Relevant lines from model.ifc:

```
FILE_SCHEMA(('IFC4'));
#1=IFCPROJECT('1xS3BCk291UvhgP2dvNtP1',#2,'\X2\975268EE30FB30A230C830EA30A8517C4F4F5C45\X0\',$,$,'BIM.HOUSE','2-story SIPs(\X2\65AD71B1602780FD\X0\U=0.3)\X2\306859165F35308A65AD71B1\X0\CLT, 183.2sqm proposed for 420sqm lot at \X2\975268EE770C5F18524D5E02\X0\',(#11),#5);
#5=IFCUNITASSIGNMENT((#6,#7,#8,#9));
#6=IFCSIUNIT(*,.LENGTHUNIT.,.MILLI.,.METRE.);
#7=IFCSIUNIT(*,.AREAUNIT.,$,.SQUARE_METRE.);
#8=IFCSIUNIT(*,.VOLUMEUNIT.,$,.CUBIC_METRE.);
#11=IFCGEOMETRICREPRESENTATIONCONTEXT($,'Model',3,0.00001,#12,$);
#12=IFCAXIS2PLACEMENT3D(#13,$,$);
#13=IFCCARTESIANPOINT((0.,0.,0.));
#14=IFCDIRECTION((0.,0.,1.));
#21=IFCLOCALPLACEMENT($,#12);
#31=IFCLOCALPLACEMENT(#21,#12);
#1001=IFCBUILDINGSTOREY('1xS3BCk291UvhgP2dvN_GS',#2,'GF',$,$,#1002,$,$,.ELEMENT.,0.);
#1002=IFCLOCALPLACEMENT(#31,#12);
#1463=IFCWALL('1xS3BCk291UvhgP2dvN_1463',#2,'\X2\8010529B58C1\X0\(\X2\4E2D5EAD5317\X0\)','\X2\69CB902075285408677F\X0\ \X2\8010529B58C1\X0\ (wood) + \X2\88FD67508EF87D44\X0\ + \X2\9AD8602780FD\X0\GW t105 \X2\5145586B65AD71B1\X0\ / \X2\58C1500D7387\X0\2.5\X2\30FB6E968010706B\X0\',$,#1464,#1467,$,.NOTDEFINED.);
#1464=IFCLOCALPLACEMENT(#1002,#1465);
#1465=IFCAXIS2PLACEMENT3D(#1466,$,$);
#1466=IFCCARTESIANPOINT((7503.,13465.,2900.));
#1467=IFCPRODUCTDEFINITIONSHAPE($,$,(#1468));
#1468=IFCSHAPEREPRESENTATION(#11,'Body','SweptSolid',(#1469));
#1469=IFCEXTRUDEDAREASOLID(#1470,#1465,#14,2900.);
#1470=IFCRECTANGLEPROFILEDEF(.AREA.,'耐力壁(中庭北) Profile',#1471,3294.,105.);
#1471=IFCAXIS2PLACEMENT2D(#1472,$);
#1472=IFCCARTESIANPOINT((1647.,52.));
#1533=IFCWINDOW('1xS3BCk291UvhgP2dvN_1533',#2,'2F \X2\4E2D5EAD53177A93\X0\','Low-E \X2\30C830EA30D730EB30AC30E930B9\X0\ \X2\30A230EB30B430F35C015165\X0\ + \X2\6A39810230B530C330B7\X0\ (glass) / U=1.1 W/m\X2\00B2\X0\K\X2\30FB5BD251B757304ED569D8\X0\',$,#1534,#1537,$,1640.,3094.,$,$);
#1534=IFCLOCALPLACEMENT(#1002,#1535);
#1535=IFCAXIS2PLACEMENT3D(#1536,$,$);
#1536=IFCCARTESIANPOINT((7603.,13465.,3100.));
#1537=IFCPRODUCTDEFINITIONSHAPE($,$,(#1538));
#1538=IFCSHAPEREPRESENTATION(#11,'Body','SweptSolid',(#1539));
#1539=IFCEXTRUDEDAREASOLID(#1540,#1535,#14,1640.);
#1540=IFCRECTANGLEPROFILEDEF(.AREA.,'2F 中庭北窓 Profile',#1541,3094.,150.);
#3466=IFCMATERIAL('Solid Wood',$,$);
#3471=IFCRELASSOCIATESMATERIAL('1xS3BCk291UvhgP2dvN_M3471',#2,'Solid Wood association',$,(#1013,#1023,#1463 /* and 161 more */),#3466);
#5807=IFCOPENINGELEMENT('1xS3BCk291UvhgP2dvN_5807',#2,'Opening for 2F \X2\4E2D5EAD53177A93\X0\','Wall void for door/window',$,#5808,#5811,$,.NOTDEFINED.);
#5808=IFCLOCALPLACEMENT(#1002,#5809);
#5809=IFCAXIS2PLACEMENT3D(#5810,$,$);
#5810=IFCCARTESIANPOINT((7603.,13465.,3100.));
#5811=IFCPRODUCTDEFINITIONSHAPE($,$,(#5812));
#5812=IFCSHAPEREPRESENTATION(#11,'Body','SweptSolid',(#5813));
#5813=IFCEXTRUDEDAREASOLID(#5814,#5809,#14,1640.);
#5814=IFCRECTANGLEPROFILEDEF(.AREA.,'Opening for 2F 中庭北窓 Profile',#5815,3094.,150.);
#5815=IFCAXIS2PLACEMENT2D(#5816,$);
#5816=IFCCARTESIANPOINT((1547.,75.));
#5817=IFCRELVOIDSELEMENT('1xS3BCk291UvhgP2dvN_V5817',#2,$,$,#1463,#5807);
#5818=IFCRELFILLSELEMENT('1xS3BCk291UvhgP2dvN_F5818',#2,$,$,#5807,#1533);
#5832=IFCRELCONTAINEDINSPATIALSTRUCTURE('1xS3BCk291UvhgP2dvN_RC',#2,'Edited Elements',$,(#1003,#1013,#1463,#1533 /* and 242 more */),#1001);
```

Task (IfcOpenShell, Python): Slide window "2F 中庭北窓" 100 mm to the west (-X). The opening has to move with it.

```python
import ifcopenshell
import ifcopenshell.api.geometry
import ifcopenshell.util.placement
import ifcopenshell.util.unit

model = ifcopenshell.open("model.ifc")
unit_scale = ifcopenshell.util.unit.calculate_unit_scale(model)

window = model.by_guid("1xS3BCk291UvhgP2dvN_1533")
opening = window.FillsVoids[0].RelatingOpeningElement
wall = opening.VoidsElements[0].RelatingBuildingElement

wall_matrix = ifcopenshell.util.placement.get_local_placement(wall.ObjectPlacement)
shift = wall_matrix[:3, 0] * -0.1 / unit_scale
before = ifcopenshell.util.placement.get_local_placement(window.ObjectPlacement)[:3, 3].copy()

# The window is not placed relative to its opening, so move both.
for product in (opening, window):
    matrix = ifcopenshell.util.placement.get_local_placement(product.ObjectPlacement)
    matrix[:3, 3] += shift
    ifcopenshell.api.geometry.edit_object_placement(model, product=product, matrix=matrix, is_si=False)

after = ifcopenshell.util.placement.get_local_placement(window.ObjectPlacement)[:3, 3]
print("window moved by", (after - before).round(3) + 0.0)

model.write("model_v2.ifc")
```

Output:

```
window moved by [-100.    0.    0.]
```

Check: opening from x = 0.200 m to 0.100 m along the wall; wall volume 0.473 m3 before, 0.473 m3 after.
